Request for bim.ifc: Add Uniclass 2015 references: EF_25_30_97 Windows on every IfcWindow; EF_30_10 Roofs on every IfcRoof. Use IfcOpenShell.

First a look at what the model holds.

```python
import ifcopenshell

model = ifcopenshell.open("bim.ifc")
print(model.schema)
print("classifications:", [c.Name for c in model.by_type("IfcClassification")])
for ifc_class in ("IfcDoor", "IfcRoof", "IfcStair", "IfcWall", "IfcWindow"):
    print(ifc_class, len(model.by_type(ifc_class)))
```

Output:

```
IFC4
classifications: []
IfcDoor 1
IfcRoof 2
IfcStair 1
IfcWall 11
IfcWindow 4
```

```python
import ifcopenshell
import ifcopenshell.api.classification

model = ifcopenshell.open("bim.ifc")

system = ifcopenshell.api.classification.add_classification(model, classification="Uniclass 2015")

codes = {
    "IfcWindow": ("EF_25_30_97", "Windows"),
    "IfcRoof": ("EF_30_10", "Roofs"),
}
for ifc_class, (code, name) in codes.items():
    products = model.by_type(ifc_class)
    ifcopenshell.api.classification.add_reference(
        model, products=products, classification=system, identification=code, name=name
    )
    print(code, len(products))

model.write("bim-out.ifc")
```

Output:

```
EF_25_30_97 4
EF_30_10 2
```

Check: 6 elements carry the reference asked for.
